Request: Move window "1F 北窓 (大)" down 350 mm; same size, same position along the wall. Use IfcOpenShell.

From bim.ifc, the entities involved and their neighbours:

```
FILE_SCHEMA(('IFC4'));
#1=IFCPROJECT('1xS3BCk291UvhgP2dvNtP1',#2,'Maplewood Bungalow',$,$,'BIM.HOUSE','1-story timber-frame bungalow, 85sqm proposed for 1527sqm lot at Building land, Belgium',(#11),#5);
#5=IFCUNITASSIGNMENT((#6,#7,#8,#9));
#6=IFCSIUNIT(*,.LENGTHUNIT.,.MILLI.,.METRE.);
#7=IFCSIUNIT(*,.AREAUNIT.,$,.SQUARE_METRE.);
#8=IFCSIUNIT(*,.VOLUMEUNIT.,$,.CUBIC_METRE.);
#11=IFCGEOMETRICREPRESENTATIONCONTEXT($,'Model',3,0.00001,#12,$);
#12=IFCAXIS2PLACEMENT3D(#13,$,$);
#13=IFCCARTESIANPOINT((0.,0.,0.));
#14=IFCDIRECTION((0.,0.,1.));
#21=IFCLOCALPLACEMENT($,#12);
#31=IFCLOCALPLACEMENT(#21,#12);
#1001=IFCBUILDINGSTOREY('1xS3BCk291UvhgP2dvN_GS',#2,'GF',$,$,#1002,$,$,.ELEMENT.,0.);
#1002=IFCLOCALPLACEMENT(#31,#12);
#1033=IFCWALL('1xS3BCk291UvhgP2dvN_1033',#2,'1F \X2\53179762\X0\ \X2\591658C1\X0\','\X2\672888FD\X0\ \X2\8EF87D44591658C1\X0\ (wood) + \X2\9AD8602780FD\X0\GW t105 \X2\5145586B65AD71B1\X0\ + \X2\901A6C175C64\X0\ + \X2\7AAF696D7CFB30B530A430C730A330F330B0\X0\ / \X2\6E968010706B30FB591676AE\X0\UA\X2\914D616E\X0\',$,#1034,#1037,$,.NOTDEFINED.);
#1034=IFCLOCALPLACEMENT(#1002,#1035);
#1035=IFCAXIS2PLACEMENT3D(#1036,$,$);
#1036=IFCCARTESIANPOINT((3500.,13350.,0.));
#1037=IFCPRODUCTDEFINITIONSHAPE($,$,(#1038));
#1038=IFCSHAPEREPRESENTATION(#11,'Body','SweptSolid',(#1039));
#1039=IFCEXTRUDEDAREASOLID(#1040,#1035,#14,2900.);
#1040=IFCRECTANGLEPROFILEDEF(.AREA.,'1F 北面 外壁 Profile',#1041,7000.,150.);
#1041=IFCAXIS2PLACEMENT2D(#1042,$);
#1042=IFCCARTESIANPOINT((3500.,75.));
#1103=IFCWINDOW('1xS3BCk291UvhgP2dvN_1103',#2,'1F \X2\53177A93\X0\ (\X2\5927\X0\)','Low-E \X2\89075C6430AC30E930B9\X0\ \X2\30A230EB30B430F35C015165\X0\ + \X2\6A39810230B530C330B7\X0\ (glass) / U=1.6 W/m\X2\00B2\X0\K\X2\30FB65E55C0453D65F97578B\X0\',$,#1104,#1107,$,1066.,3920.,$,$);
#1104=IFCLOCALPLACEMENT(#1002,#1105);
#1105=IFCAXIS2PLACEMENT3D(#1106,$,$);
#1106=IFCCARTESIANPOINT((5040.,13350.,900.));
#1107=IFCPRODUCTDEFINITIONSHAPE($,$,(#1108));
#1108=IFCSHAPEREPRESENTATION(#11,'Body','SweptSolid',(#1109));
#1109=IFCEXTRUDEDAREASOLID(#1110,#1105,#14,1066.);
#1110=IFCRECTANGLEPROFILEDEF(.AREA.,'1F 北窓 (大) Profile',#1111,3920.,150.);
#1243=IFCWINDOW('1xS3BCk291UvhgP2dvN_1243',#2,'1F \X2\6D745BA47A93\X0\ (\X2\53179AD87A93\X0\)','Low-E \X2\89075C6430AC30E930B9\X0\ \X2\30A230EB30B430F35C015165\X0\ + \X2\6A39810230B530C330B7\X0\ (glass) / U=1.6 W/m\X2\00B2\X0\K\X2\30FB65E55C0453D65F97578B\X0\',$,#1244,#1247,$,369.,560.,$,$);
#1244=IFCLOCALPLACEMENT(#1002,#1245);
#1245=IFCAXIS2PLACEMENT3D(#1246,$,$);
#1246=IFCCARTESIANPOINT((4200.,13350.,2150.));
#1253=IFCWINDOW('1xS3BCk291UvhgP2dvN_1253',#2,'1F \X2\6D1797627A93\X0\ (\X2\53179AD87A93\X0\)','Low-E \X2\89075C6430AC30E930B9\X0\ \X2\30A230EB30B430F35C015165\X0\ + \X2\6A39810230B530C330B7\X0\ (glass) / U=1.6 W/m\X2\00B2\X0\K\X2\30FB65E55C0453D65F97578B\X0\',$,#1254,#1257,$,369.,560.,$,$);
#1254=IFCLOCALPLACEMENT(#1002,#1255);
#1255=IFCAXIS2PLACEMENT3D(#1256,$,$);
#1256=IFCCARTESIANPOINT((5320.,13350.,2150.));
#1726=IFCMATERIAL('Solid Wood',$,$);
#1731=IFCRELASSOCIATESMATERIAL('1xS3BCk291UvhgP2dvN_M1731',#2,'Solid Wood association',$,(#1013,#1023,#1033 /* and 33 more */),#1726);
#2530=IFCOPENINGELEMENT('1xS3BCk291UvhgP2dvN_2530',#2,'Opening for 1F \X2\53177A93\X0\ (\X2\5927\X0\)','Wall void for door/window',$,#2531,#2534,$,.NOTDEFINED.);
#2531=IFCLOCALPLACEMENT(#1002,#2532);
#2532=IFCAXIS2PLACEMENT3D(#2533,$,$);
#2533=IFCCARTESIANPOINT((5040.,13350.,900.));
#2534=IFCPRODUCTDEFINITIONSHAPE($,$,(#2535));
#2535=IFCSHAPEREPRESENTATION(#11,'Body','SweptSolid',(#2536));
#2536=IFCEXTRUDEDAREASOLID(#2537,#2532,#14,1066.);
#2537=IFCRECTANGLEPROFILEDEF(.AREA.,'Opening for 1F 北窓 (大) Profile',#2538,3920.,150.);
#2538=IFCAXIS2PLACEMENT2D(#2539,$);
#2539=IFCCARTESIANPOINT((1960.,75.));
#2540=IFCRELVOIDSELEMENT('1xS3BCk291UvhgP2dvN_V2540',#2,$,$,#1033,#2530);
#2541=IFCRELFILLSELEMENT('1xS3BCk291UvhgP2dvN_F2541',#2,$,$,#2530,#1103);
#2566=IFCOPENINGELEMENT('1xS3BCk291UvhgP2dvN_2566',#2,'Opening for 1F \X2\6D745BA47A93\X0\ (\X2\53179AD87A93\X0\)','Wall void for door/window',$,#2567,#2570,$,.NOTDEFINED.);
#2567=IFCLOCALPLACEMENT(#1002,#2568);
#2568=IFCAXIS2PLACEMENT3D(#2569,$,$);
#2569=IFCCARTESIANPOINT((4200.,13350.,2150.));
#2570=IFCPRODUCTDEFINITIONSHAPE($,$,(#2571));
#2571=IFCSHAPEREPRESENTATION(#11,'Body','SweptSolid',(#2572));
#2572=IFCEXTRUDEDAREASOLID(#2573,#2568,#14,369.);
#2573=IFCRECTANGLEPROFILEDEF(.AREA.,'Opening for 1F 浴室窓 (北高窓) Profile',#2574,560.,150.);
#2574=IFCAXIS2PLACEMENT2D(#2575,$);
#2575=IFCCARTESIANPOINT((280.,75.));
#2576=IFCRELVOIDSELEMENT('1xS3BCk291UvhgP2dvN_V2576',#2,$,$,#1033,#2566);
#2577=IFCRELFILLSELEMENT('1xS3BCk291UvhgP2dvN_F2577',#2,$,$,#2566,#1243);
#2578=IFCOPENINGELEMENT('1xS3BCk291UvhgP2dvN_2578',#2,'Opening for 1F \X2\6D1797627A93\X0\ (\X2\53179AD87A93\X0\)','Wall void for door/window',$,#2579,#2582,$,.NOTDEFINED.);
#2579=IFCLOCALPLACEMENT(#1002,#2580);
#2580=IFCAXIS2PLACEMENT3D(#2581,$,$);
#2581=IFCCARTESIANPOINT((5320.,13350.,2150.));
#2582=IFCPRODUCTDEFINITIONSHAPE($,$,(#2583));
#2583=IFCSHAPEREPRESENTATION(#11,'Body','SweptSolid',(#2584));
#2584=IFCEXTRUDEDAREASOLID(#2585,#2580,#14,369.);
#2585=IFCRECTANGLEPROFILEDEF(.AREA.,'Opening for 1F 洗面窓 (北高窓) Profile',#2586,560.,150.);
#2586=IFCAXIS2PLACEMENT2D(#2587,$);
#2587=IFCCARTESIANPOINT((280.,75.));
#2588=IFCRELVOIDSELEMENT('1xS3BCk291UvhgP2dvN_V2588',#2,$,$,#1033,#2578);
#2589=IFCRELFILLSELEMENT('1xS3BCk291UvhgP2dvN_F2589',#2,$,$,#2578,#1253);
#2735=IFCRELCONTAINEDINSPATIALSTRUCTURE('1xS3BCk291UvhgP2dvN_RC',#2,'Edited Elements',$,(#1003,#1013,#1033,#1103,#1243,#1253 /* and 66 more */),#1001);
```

```python
import numpy as np
import ifcopenshell
import ifcopenshell.api.geometry
import ifcopenshell.util.placement
import ifcopenshell.util.unit

model = ifcopenshell.open("bim.ifc")
unit_scale = ifcopenshell.util.unit.calculate_unit_scale(model)

window = model.by_id(1103)
opening = window.FillsVoids[0].RelatingOpeningElement
dz = -350.0

shift = np.array([0.0, 0.0, dz])
# The window is not placed relative to its opening, so move both.
for product in (opening, window):
    matrix = ifcopenshell.util.placement.get_local_placement(product.ObjectPlacement)
    matrix[:3, 3] += shift
    ifcopenshell.api.geometry.edit_object_placement(model, product=product, matrix=matrix, is_si=False)

print(f"moved by {dz * unit_scale:+.3f} m")

model.write("bim_v2.ifc")
```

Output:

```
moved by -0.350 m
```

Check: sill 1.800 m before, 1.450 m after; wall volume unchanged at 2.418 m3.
